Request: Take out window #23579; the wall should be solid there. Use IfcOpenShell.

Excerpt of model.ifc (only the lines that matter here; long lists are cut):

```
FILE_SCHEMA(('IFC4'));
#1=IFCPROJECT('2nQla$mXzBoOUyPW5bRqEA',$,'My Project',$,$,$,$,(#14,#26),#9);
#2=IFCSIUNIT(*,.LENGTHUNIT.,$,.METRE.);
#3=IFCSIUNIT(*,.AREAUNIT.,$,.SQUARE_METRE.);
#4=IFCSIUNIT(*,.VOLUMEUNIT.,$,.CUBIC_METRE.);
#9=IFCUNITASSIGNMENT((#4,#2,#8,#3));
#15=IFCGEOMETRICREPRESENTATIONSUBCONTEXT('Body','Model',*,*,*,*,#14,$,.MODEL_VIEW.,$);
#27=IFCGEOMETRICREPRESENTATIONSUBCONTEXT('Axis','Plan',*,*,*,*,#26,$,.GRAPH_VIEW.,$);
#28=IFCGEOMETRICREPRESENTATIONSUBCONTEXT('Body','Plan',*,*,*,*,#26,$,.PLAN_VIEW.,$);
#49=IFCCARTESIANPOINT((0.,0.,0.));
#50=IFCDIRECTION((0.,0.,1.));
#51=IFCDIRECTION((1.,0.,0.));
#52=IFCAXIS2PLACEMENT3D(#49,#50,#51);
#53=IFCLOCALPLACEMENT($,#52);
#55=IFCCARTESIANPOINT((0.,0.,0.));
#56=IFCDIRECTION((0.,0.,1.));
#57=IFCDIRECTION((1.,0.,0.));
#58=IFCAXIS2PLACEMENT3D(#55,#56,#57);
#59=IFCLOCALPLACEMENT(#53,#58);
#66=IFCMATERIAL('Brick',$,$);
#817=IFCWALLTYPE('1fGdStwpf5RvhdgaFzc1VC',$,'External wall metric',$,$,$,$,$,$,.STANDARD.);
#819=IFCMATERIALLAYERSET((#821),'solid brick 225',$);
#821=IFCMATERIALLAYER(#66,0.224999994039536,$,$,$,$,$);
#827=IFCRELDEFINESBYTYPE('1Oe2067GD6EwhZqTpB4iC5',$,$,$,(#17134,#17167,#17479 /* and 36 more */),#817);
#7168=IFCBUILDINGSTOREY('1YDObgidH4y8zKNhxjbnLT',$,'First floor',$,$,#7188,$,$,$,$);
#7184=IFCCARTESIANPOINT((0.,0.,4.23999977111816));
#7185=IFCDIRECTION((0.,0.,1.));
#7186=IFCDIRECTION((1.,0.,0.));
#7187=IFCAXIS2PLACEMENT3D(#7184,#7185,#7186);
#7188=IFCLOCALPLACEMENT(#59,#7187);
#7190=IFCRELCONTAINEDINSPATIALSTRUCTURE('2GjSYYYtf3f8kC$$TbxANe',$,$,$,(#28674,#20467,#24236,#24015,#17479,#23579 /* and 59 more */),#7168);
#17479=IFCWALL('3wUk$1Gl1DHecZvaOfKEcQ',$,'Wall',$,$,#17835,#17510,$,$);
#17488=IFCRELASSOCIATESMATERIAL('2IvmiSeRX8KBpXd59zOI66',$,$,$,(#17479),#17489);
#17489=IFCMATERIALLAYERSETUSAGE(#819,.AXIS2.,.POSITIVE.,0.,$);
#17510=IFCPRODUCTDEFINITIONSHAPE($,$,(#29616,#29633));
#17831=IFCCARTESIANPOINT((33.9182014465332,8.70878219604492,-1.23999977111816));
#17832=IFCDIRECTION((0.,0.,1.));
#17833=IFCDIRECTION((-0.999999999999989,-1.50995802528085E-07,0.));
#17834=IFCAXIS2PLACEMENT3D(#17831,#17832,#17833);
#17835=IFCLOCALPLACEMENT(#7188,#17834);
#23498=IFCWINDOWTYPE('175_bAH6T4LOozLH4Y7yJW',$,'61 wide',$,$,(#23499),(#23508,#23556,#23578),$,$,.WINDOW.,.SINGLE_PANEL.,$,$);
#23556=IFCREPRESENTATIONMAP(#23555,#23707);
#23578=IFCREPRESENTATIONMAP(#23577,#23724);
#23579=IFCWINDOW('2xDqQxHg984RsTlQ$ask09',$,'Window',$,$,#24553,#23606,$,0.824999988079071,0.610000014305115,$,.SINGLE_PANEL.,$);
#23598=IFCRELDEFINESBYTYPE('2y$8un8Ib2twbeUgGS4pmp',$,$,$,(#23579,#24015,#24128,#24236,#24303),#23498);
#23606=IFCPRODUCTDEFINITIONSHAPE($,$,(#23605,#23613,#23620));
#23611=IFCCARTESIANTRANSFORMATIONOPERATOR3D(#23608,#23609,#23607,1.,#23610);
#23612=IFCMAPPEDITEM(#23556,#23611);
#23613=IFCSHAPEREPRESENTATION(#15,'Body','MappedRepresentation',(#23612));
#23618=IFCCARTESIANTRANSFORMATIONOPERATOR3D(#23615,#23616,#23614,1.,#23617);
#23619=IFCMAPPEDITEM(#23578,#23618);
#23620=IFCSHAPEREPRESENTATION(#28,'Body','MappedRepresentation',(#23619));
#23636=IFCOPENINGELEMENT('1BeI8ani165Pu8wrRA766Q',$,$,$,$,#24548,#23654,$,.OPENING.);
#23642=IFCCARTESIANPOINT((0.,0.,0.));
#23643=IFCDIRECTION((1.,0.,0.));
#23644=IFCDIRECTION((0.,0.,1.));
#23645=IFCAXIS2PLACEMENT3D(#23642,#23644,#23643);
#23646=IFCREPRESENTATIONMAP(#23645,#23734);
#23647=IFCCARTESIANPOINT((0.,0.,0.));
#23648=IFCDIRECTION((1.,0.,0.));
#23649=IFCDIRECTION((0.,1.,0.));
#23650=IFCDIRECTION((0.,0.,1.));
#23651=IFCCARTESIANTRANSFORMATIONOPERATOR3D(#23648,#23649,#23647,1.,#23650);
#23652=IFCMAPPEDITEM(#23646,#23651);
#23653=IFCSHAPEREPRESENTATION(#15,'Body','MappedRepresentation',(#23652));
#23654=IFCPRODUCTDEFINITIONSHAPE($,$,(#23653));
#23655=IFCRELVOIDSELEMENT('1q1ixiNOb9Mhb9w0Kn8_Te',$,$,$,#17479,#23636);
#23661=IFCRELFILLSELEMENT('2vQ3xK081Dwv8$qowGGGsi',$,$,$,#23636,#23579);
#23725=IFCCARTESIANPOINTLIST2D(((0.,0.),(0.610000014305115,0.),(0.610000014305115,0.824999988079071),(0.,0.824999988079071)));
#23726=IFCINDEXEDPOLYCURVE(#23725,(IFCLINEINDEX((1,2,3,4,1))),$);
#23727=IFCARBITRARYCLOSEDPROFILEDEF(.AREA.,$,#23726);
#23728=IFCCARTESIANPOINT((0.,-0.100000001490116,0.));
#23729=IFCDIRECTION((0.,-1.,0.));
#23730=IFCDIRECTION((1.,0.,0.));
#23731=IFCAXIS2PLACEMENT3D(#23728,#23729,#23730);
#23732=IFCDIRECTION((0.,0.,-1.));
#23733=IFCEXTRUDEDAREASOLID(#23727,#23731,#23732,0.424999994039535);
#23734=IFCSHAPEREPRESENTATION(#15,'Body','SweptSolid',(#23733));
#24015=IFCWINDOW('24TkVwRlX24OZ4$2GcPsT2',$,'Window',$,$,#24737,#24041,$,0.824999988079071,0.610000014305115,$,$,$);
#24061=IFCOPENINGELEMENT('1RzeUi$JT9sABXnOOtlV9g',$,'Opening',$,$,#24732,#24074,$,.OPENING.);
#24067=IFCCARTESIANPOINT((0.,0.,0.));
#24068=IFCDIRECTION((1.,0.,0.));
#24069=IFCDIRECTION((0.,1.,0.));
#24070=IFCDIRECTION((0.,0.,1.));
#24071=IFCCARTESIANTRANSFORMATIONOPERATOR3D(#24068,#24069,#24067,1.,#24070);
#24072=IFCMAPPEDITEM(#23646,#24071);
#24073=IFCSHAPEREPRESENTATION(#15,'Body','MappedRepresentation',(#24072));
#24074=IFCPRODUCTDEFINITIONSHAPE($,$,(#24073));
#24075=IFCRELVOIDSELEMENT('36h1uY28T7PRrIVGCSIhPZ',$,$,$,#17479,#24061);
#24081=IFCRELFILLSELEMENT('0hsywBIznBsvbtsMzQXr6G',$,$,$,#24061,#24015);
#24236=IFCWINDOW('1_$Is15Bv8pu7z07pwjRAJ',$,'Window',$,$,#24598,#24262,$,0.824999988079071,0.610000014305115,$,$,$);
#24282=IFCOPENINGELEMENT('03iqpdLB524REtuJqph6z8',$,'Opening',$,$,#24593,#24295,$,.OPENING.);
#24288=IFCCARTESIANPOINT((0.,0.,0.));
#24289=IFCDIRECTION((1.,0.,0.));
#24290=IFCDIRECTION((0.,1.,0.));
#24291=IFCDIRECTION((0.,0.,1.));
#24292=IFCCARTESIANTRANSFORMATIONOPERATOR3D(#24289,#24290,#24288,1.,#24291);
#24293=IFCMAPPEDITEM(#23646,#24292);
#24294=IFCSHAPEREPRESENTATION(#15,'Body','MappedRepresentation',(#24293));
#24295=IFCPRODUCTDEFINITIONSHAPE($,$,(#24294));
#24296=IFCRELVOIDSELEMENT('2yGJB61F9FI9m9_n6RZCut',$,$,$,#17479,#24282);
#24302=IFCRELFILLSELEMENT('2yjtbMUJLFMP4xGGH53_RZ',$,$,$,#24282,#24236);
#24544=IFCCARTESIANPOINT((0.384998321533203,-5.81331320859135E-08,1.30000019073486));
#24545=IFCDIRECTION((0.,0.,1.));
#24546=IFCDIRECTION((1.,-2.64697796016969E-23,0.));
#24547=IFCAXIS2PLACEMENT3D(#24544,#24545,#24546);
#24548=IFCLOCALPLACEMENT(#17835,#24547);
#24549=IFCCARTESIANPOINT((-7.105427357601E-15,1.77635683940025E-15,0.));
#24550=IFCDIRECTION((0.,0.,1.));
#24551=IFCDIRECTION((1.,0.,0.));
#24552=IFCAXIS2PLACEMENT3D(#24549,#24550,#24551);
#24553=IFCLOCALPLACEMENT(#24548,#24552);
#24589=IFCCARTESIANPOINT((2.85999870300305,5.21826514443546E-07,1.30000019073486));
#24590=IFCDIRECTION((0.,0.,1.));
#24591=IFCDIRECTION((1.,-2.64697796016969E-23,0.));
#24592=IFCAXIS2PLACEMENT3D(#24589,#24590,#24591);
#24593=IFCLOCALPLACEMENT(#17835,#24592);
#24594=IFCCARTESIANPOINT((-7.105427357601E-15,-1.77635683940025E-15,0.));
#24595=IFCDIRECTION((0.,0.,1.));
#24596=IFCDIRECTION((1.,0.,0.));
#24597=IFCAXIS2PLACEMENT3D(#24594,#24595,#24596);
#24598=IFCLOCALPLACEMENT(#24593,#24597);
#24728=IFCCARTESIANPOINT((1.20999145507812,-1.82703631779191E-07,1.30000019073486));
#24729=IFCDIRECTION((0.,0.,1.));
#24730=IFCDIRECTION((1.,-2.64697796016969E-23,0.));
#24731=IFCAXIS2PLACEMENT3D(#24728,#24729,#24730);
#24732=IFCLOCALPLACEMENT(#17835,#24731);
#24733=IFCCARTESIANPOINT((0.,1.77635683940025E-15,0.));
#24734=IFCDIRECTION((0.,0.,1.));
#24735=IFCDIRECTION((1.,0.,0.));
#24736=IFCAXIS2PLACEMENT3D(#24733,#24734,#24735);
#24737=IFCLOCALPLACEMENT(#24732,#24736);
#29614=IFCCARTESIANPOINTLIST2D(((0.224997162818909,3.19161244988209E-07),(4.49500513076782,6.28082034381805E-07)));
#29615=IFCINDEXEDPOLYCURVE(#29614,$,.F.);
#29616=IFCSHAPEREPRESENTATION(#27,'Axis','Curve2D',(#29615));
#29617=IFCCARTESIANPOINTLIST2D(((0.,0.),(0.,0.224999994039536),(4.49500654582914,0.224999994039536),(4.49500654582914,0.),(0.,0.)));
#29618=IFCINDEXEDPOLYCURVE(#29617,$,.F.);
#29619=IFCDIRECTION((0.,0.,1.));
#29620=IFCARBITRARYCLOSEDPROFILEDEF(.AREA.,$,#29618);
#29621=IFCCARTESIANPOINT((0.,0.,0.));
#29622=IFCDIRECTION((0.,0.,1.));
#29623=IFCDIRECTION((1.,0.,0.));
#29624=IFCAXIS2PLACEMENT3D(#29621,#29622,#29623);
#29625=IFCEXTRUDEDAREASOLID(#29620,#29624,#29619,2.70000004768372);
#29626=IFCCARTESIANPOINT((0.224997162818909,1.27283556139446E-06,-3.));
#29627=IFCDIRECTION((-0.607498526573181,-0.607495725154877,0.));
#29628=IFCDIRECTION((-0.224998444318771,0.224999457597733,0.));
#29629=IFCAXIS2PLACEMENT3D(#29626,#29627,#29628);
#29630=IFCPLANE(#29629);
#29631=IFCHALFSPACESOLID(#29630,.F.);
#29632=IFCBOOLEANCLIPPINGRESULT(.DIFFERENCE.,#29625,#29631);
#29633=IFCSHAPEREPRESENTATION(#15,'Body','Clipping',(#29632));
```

```python
import ifcopenshell
import ifcopenshell.api.feature
import ifcopenshell.api.root
import ifcopenshell.geom
import ifcopenshell.util.shape

model = ifcopenshell.open("model.ifc")
settings = ifcopenshell.geom.settings()


def volume(element):
    """Net volume in cubic metres, openings subtracted."""
    shape = ifcopenshell.geom.create_shape(settings, element)
    return ifcopenshell.util.shape.get_volume(shape.geometry)


window = model.by_guid("2xDqQxHg984RsTlQ$ask09")
opening = window.FillsVoids[0].RelatingOpeningElement
wall = opening.VoidsElements[0].RelatingBuildingElement
before = volume(wall)

ifcopenshell.api.root.remove_product(model, product=window)
ifcopenshell.api.feature.remove_feature(model, feature=opening)

after = volume(wall)

print(f"wall volume {before:.3f} -> {after:.3f} m3")

model.write("model_updated.ifc")
```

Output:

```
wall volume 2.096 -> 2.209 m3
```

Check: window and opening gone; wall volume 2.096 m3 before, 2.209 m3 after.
